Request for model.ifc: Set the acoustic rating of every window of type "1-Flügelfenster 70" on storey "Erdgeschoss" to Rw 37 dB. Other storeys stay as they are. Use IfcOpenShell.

First a look at what the model holds.

```python
import ifcopenshell
import ifcopenshell.util.element

model = ifcopenshell.open("model.ifc")
print(model.schema)
storey = next(s for s in model.by_type("IfcBuildingStorey") if s.Name == "Erdgeschoss")
windows = [e for e in ifcopenshell.util.element.get_decomposition(storey) if e.is_a("IfcWindow")]
seen = {}
for e in windows:
    element_type = ifcopenshell.util.element.get_type(e)
    key = (element_type.Name if element_type != e and element_type else None, ifcopenshell.util.element.get_pset(e, "Pset_WindowCommon", "AcousticRating"))
    seen[key] = seen.get(key, 0) + 1
for (name, value), count in sorted(seen.items(), key=str):
    print(count, "x", name, "|", value)
```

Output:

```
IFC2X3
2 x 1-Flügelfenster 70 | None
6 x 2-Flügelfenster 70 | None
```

```python
import ifcopenshell
import ifcopenshell.api.pset
import ifcopenshell.util.element

model = ifcopenshell.open("model.ifc")

storey = next(s for s in model.by_type("IfcBuildingStorey") if s.Name == "Erdgeschoss")
windows = [e for e in ifcopenshell.util.element.get_decomposition(storey) if e.is_a("IfcWindow")]

count = 0
for e in windows:
    element_type = ifcopenshell.util.element.get_type(e)
    if element_type in (None, e) or element_type.Name != "1-Flügelfenster 70":
        continue
    # add_pset returns the element's existing set when there is one.
    pset = ifcopenshell.api.pset.add_pset(model, product=e, name="Pset_WindowCommon")
    ifcopenshell.api.pset.edit_pset(model, pset=pset, properties={"AcousticRating": "Rw 37 dB"})
    count += 1

print(count, "windows updated")

model.write("model-out.ifc")
```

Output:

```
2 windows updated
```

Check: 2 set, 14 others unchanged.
